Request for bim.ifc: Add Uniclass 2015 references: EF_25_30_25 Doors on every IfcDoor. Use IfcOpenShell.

First a look at what the model holds.

```python
import ifcopenshell

model = ifcopenshell.open("bim.ifc")
print(model.schema)
print("classifications:", [c.Name for c in model.by_type("IfcClassification")])
for ifc_class in ("IfcDoor", "IfcRoof", "IfcStair", "IfcWall", "IfcWindow"):
    print(ifc_class, len(model.by_type(ifc_class)))
```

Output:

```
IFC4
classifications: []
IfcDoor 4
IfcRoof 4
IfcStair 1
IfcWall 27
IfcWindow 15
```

```python
import ifcopenshell
import ifcopenshell.api.classification

model = ifcopenshell.open("bim.ifc")

system = ifcopenshell.api.classification.add_classification(model, classification="Uniclass 2015")

codes = {
    "IfcDoor": ("EF_25_30_25", "Doors"),
}
for ifc_class, (code, name) in codes.items():
    products = model.by_type(ifc_class)
    ifcopenshell.api.classification.add_reference(
        model, products=products, classification=system, identification=code, name=name
    )
    print(code, len(products))

model.write("bim_updated.ifc")
```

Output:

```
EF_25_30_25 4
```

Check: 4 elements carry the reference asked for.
